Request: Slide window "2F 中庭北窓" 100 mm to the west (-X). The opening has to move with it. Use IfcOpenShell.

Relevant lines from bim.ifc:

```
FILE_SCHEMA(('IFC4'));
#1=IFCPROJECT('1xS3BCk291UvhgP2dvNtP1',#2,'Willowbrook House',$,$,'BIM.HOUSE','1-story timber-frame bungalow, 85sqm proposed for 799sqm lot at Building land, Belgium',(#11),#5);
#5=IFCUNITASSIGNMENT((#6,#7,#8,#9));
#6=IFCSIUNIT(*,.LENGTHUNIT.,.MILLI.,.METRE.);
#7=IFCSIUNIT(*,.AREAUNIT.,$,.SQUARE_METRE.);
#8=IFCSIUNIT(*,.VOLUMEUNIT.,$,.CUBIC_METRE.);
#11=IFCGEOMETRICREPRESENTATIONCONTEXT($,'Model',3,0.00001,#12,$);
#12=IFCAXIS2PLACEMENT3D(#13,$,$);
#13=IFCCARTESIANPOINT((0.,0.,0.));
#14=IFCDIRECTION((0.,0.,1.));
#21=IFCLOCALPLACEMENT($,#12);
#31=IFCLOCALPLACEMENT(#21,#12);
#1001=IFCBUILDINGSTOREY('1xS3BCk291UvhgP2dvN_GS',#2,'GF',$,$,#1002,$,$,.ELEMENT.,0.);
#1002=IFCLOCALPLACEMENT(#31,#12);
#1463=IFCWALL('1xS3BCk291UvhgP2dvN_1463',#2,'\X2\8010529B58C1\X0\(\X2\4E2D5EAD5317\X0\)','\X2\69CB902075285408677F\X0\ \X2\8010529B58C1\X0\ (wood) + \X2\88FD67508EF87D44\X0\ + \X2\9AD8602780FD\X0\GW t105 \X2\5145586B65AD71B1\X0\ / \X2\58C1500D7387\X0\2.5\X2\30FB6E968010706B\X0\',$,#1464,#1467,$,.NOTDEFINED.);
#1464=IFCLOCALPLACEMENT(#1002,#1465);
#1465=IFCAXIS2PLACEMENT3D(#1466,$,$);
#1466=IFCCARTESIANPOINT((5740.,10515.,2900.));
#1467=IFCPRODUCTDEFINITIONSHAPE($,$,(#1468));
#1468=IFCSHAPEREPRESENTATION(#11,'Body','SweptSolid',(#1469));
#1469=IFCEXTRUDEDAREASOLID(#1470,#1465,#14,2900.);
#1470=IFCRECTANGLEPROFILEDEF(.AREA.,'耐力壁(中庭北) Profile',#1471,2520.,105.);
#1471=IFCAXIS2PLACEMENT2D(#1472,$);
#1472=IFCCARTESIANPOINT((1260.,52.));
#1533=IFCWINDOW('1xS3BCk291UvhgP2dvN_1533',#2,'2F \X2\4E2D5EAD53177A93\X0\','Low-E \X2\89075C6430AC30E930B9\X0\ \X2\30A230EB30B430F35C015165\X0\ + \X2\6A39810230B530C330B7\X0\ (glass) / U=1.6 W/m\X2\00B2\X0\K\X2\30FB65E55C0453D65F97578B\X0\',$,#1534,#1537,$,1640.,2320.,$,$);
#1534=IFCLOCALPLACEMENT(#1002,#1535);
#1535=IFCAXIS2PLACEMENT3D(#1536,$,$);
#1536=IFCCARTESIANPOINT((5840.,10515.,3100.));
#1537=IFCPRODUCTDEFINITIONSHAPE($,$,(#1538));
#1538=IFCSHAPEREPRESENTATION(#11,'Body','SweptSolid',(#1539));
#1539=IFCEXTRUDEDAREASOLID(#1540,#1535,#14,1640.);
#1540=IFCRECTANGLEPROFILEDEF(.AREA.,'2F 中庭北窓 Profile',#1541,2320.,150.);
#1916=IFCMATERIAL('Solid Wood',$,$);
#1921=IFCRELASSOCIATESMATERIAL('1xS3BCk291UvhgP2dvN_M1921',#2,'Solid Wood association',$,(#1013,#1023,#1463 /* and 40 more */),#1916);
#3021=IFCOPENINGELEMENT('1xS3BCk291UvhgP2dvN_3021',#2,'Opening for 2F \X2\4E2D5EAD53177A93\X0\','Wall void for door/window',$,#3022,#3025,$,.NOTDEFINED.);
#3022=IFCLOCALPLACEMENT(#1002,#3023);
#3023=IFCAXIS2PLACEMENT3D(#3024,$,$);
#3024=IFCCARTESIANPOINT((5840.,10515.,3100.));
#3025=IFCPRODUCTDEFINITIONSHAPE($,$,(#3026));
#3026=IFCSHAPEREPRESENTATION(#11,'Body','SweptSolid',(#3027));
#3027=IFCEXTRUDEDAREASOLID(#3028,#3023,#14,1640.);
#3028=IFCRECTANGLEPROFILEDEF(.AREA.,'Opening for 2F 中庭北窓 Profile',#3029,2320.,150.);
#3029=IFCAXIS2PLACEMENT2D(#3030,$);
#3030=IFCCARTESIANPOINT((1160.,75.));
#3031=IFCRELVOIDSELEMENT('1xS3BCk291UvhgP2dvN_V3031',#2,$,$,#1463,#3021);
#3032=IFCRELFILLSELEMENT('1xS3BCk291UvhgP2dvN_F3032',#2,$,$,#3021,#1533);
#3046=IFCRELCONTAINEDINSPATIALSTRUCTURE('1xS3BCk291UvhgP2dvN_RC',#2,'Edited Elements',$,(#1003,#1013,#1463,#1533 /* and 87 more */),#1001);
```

```python
import ifcopenshell
import ifcopenshell.api.geometry
import ifcopenshell.util.placement

model = ifcopenshell.open("bim.ifc")

window = model.by_guid("1xS3BCk291UvhgP2dvN_1533")
opening = window.FillsVoids[0].RelatingOpeningElement
wall = opening.VoidsElements[0].RelatingBuildingElement

wall_matrix = ifcopenshell.util.placement.get_local_placement(wall.ObjectPlacement)
shift = wall_matrix[:3, 0] * -100.0
before = ifcopenshell.util.placement.get_local_placement(window.ObjectPlacement)[:3, 3].copy()

# The window is not placed relative to its opening, so move both.
for product in (opening, window):
    matrix = ifcopenshell.util.placement.get_local_placement(product.ObjectPlacement)
    matrix[:3, 3] += shift
    ifcopenshell.api.geometry.edit_object_placement(model, product=product, matrix=matrix, is_si=False)

after = ifcopenshell.util.placement.get_local_placement(window.ObjectPlacement)[:3, 3]
print("window moved by", (after - before).round(3) + 0.0)

model.write("bim-out.ifc")
```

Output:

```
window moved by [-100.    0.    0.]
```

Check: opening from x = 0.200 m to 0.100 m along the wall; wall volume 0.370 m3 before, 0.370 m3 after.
